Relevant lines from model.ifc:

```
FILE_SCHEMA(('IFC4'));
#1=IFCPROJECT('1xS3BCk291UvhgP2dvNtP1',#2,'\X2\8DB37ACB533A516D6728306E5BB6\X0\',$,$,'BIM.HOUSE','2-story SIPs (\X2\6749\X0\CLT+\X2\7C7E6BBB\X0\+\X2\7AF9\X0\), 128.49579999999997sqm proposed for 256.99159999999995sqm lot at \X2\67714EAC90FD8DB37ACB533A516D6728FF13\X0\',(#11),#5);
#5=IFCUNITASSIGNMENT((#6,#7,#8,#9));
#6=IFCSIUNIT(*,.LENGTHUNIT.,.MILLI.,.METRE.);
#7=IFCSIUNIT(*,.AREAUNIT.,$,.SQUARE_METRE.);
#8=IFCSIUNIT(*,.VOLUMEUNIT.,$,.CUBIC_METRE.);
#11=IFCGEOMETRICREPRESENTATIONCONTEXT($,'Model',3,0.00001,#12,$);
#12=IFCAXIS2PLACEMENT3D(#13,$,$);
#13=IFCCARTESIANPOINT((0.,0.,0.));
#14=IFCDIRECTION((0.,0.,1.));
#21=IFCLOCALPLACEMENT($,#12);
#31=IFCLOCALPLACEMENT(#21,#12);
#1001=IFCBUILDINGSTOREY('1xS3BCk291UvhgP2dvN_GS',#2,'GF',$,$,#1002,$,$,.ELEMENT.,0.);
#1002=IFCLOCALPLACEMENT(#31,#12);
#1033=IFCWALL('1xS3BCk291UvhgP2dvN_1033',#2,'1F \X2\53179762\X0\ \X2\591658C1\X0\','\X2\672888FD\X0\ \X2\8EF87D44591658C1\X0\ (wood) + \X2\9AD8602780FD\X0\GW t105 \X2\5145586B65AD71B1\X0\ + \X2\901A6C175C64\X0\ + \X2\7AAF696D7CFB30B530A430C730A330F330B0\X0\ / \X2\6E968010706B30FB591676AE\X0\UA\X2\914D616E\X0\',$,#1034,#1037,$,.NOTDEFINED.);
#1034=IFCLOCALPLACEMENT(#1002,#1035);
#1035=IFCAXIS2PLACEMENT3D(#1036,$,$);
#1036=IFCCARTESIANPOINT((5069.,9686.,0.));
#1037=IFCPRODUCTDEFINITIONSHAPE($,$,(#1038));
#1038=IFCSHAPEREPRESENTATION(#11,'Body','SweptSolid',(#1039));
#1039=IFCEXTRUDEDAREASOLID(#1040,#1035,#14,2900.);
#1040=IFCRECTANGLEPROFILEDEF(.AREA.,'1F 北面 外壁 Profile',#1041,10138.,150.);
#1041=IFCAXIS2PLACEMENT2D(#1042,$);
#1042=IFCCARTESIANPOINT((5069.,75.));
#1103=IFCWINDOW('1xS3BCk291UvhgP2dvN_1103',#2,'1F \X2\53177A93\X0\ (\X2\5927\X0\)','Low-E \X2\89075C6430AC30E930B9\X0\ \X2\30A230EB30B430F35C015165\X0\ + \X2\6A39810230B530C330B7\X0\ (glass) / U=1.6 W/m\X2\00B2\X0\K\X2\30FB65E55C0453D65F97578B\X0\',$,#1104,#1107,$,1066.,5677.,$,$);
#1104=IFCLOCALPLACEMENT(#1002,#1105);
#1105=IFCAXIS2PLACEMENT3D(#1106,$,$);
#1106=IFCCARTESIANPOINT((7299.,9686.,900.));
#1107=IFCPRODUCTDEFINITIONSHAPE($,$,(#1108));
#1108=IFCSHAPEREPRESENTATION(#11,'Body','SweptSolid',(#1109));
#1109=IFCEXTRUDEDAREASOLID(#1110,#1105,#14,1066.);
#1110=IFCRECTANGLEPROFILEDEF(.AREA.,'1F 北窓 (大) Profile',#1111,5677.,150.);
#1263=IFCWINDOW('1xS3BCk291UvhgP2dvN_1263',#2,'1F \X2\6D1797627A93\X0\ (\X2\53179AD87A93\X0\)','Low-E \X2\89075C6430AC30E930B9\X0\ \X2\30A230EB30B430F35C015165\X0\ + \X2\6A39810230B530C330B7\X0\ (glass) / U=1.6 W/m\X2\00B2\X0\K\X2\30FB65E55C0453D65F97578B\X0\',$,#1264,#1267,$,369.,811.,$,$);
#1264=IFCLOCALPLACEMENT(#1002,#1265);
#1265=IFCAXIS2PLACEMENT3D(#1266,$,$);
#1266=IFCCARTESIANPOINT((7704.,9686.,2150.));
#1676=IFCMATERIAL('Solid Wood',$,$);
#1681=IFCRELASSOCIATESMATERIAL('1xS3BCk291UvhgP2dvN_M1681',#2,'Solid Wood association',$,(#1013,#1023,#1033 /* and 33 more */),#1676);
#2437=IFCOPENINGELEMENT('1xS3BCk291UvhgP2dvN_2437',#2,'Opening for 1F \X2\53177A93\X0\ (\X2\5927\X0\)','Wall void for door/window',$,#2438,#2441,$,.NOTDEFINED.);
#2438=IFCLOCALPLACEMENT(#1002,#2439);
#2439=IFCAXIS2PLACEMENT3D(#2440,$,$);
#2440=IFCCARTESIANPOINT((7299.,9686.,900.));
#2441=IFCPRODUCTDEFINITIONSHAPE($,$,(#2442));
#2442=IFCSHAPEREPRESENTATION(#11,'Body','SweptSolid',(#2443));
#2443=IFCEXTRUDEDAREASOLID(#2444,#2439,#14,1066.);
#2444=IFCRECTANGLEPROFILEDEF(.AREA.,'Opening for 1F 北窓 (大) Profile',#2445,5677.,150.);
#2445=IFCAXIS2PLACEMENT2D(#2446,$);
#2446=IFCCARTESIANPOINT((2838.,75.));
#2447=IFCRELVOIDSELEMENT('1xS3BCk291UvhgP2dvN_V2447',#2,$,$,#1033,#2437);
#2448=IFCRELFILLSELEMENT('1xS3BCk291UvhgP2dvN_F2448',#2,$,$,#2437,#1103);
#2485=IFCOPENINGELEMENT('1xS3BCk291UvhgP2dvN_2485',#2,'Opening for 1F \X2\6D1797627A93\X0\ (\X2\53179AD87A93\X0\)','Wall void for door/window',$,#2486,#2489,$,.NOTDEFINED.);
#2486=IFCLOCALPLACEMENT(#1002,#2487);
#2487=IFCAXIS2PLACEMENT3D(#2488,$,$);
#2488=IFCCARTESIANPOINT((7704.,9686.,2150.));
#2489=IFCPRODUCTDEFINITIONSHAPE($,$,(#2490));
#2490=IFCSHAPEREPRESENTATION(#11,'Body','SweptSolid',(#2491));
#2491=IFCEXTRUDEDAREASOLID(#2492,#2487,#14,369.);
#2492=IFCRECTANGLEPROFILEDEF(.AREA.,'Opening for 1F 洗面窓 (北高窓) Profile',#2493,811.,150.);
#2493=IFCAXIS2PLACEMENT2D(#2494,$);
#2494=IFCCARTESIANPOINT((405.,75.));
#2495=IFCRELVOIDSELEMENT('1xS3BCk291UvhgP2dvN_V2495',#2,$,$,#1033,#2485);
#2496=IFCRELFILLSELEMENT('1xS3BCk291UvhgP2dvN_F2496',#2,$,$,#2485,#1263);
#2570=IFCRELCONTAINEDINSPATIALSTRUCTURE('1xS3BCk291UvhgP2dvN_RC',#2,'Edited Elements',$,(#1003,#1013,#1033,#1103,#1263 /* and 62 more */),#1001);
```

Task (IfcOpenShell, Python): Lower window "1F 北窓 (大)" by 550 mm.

```python
import numpy as np
import ifcopenshell
import ifcopenshell.api.geometry
import ifcopenshell.util.placement
import ifcopenshell.util.unit

model = ifcopenshell.open("model.ifc")
unit_scale = ifcopenshell.util.unit.calculate_unit_scale(model)

window = model.by_guid("1xS3BCk291UvhgP2dvN_1103")
opening = window.FillsVoids[0].RelatingOpeningElement
dz = -550.0

shift = np.array([0.0, 0.0, dz])
# The window is not placed relative to its opening, so move both.
for product in (opening, window):
    matrix = ifcopenshell.util.placement.get_local_placement(product.ObjectPlacement)
    matrix[:3, 3] += shift
    ifcopenshell.api.geometry.edit_object_placement(model, product=product, matrix=matrix, is_si=False)

print(f"moved by {dz * unit_scale:+.3f} m")

model.write("model_rev.ifc")
```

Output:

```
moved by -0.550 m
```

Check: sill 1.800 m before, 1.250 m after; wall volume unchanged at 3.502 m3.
